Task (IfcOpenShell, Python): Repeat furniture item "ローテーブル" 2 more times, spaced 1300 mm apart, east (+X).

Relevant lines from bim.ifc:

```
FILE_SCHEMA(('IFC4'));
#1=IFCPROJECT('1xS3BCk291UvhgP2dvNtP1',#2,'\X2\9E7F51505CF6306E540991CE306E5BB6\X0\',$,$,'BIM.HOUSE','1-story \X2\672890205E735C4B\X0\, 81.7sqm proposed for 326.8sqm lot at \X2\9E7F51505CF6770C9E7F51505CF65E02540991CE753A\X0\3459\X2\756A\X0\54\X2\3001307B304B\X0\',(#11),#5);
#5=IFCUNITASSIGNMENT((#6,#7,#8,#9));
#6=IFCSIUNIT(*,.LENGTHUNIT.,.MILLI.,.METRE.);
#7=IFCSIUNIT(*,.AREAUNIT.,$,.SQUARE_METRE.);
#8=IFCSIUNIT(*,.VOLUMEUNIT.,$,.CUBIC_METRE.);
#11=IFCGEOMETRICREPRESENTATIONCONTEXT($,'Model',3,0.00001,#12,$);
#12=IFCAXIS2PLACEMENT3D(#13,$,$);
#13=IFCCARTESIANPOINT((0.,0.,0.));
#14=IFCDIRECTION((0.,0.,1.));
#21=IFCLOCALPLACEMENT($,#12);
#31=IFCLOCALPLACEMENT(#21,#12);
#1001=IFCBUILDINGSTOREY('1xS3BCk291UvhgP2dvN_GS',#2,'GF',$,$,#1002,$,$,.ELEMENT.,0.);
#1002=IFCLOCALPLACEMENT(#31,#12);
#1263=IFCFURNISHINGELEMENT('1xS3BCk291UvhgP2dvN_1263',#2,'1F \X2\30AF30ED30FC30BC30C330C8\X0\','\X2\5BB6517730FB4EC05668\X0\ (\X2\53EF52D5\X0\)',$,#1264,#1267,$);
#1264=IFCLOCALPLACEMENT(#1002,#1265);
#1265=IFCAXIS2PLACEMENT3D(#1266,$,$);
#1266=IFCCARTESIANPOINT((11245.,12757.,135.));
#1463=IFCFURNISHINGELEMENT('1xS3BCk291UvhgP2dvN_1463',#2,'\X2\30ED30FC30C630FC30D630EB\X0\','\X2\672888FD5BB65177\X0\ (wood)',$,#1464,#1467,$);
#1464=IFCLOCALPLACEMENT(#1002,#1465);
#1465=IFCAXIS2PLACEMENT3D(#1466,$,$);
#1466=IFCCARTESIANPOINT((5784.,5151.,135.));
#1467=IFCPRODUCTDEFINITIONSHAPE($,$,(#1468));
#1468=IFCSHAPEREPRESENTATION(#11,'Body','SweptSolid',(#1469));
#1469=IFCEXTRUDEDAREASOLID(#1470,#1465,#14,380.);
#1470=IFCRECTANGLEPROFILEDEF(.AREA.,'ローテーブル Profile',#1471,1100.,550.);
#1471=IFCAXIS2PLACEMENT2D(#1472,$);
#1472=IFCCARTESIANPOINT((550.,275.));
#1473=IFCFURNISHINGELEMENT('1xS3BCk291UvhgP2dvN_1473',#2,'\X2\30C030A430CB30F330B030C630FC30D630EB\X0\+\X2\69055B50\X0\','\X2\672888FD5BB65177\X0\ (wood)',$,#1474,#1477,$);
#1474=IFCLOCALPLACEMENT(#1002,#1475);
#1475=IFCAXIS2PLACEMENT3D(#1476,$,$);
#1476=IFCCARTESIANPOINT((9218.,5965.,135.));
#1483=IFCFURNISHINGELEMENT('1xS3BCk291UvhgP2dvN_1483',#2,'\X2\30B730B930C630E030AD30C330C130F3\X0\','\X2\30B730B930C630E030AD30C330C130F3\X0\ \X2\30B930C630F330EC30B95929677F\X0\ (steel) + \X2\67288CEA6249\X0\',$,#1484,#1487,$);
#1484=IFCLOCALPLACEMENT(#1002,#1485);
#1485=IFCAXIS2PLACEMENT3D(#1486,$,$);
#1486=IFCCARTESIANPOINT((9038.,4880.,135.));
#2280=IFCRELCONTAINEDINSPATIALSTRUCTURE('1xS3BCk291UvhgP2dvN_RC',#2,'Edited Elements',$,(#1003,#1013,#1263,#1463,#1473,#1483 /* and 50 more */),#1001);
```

```python
import numpy as np
import ifcopenshell
import ifcopenshell.api.geometry
import ifcopenshell.api.root
import ifcopenshell.util.element
import ifcopenshell.util.placement

model = ifcopenshell.open("bim.ifc")


def reuse_history(source, copy):
    """copy_class also copies each property set's owner history, people and application; keep the originals."""
    for rel in copy.IsDefinedBy:
        if rel.is_a("IfcRelDefinesByProperties") and (history := rel.RelatingPropertyDefinition.OwnerHistory):
            rel.RelatingPropertyDefinition.OwnerHistory = source.OwnerHistory
            ifcopenshell.util.element.remove_deep2(model, history)


source = model.by_id(1463)
base = ifcopenshell.util.placement.get_local_placement(source.ObjectPlacement)
step = np.array([1.0, 0.0, 0.0]) * 1300.0

for i in range(1, 3):
    copy = ifcopenshell.api.root.copy_class(model, product=source)
    copy.Representation = ifcopenshell.util.element.copy_deep(
        model, source.Representation, exclude=["IfcGeometricRepresentationContext", "IfcRepresentationMap"]
    )
    reuse_history(source, copy)
    matrix = base.copy()
    matrix[:3, 3] += i * step
    print("added at", matrix[:3, 3].round(3) + 0.0)
    ifcopenshell.api.geometry.edit_object_placement(model, product=copy, matrix=matrix, is_si=False)

model.write("bim_updated.ifc")
```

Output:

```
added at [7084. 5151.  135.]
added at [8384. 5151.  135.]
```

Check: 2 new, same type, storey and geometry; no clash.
